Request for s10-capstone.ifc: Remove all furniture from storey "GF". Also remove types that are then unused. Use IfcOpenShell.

First a look at what the model holds.

```python
import ifcopenshell
import ifcopenshell.util.element

model = ifcopenshell.open("s10-capstone.ifc")
print(model.schema)
storey = next(s for s in model.by_type("IfcBuildingStorey") if s.Name == "GF")
furniture = [e for e in ifcopenshell.util.element.get_decomposition(storey) if e.is_a("IfcFurnishingElement")]
seen = {}
for e in furniture:
    element_type = ifcopenshell.util.element.get_type(e)
    name = element_type.Name if element_type not in (None, e) else None
    seen[name] = seen.get(name, 0) + 1
for name, count in sorted(seen.items(), key=str):
    print(count, "x", name)
```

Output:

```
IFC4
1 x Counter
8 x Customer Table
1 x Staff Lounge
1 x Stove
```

```python
import ifcopenshell
import ifcopenshell.api.root
import ifcopenshell.util.element

model = ifcopenshell.open("s10-capstone.ifc")

storey = next(s for s in model.by_type("IfcBuildingStorey") if s.Name == "GF")
furniture = [e for e in ifcopenshell.util.element.get_decomposition(storey) if e.is_a("IfcFurnishingElement")]
types = {ifcopenshell.util.element.get_type(e) for e in furniture} - {None, *furniture}

for e in furniture:
    ifcopenshell.api.root.remove_product(model, product=e)
print(len(furniture), "removed")

unused = [t for t in types if not ifcopenshell.util.element.get_types(t)]
for t in unused:
    ifcopenshell.api.root.remove_product(model, product=t)
print(len(unused), "unused types removed")

model.write("s10-capstone_rev.ifc")
```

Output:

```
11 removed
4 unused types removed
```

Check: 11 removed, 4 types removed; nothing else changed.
